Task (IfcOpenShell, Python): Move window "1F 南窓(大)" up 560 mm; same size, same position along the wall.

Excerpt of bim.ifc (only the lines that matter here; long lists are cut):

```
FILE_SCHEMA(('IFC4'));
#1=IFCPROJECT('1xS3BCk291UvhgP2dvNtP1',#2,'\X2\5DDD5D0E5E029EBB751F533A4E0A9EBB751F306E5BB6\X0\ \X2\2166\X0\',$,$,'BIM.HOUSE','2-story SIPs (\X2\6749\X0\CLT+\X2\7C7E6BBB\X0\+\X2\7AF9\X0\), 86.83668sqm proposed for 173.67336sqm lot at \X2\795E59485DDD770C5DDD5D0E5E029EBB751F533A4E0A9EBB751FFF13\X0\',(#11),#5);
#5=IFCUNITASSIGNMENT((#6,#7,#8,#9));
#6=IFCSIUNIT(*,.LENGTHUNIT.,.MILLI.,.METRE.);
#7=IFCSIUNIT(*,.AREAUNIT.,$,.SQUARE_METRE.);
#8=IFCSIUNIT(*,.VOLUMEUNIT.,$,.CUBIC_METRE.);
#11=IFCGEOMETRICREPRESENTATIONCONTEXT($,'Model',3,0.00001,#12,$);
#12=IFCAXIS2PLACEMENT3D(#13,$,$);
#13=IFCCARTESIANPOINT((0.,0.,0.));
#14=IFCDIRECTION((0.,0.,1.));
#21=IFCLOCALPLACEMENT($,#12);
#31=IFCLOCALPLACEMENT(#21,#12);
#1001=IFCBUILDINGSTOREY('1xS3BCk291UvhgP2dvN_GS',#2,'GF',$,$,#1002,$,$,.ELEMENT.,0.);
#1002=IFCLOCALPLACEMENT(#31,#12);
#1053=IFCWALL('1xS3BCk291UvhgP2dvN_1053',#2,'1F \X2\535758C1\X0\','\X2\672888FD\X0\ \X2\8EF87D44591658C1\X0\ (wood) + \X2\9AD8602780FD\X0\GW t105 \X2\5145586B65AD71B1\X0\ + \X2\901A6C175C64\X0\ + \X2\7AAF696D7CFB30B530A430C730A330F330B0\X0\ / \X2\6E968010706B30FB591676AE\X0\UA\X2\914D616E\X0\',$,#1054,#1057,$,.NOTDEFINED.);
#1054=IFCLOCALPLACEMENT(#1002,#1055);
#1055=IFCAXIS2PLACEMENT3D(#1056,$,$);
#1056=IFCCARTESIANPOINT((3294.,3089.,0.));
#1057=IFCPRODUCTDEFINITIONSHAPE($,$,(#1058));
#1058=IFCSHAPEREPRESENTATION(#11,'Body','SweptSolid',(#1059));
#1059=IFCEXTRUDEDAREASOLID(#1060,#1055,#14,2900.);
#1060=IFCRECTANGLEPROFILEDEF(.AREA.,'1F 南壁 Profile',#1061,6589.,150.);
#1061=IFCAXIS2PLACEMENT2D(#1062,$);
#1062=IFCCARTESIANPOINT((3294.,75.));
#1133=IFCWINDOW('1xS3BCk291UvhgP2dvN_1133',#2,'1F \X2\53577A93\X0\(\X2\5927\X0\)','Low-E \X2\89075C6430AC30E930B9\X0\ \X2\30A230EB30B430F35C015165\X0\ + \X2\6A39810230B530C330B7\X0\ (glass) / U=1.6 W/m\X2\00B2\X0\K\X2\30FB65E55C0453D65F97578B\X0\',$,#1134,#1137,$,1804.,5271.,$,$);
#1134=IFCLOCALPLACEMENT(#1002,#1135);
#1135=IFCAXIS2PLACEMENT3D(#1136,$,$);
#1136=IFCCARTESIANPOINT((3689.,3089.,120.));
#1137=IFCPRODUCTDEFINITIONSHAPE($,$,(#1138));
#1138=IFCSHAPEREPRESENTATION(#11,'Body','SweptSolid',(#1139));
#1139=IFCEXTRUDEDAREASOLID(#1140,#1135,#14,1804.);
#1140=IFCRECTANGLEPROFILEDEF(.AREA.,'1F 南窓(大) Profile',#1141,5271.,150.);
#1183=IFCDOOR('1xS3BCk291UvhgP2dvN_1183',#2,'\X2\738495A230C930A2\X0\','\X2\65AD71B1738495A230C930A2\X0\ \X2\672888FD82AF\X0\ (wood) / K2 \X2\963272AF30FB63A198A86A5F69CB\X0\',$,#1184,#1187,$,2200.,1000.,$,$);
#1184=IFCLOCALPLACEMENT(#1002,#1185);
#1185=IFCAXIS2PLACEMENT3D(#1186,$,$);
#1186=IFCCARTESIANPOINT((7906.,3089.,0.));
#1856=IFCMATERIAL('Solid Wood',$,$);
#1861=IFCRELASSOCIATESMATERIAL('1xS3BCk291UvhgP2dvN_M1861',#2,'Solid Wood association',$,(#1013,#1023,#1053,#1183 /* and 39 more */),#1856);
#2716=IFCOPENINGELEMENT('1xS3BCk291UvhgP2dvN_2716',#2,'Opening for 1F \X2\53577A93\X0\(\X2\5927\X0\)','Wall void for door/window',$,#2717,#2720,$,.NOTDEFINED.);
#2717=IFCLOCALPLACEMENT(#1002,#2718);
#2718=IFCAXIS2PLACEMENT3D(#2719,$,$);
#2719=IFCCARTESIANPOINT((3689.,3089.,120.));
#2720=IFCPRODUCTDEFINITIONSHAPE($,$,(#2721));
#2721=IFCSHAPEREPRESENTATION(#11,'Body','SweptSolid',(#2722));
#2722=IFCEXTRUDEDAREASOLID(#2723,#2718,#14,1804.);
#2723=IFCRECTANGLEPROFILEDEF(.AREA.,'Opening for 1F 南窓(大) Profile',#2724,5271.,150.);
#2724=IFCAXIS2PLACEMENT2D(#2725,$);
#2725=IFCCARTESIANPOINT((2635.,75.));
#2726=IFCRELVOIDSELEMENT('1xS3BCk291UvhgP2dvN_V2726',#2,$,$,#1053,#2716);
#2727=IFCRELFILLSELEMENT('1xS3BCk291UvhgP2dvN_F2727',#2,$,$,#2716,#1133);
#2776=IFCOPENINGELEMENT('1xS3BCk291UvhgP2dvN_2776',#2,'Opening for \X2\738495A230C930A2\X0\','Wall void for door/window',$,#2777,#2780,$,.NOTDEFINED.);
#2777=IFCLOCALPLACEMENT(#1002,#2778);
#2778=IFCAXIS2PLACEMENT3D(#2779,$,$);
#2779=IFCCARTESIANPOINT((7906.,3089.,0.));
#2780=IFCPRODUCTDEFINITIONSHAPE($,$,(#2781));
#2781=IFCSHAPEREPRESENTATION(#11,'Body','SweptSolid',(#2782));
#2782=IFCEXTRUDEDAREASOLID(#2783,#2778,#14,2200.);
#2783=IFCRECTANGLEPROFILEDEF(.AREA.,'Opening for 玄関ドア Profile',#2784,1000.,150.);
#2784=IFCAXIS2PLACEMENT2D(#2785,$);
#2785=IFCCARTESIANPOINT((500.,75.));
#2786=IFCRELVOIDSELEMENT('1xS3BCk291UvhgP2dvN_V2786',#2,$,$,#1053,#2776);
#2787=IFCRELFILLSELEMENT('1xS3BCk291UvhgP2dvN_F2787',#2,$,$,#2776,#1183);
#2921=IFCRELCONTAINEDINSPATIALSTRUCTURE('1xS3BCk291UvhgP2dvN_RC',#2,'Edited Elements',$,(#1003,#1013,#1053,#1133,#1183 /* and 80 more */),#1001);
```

```python
import numpy as np
import ifcopenshell
import ifcopenshell.api.geometry
import ifcopenshell.util.placement
import ifcopenshell.util.unit

model = ifcopenshell.open("bim.ifc")
unit_scale = ifcopenshell.util.unit.calculate_unit_scale(model)

window = model.by_guid("1xS3BCk291UvhgP2dvN_1133")
opening = window.FillsVoids[0].RelatingOpeningElement
dz = 0.56 / unit_scale

shift = np.array([0.0, 0.0, dz])
# The window is not placed relative to its opening, so move both.
for product in (opening, window):
    matrix = ifcopenshell.util.placement.get_local_placement(product.ObjectPlacement)
    matrix[:3, 3] += shift
    ifcopenshell.api.geometry.edit_object_placement(model, product=product, matrix=matrix, is_si=False)

print(f"moved by {dz * unit_scale:+.3f} m")

model.write("bim_v2.ifc")
```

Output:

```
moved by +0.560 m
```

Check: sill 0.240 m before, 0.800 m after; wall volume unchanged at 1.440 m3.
